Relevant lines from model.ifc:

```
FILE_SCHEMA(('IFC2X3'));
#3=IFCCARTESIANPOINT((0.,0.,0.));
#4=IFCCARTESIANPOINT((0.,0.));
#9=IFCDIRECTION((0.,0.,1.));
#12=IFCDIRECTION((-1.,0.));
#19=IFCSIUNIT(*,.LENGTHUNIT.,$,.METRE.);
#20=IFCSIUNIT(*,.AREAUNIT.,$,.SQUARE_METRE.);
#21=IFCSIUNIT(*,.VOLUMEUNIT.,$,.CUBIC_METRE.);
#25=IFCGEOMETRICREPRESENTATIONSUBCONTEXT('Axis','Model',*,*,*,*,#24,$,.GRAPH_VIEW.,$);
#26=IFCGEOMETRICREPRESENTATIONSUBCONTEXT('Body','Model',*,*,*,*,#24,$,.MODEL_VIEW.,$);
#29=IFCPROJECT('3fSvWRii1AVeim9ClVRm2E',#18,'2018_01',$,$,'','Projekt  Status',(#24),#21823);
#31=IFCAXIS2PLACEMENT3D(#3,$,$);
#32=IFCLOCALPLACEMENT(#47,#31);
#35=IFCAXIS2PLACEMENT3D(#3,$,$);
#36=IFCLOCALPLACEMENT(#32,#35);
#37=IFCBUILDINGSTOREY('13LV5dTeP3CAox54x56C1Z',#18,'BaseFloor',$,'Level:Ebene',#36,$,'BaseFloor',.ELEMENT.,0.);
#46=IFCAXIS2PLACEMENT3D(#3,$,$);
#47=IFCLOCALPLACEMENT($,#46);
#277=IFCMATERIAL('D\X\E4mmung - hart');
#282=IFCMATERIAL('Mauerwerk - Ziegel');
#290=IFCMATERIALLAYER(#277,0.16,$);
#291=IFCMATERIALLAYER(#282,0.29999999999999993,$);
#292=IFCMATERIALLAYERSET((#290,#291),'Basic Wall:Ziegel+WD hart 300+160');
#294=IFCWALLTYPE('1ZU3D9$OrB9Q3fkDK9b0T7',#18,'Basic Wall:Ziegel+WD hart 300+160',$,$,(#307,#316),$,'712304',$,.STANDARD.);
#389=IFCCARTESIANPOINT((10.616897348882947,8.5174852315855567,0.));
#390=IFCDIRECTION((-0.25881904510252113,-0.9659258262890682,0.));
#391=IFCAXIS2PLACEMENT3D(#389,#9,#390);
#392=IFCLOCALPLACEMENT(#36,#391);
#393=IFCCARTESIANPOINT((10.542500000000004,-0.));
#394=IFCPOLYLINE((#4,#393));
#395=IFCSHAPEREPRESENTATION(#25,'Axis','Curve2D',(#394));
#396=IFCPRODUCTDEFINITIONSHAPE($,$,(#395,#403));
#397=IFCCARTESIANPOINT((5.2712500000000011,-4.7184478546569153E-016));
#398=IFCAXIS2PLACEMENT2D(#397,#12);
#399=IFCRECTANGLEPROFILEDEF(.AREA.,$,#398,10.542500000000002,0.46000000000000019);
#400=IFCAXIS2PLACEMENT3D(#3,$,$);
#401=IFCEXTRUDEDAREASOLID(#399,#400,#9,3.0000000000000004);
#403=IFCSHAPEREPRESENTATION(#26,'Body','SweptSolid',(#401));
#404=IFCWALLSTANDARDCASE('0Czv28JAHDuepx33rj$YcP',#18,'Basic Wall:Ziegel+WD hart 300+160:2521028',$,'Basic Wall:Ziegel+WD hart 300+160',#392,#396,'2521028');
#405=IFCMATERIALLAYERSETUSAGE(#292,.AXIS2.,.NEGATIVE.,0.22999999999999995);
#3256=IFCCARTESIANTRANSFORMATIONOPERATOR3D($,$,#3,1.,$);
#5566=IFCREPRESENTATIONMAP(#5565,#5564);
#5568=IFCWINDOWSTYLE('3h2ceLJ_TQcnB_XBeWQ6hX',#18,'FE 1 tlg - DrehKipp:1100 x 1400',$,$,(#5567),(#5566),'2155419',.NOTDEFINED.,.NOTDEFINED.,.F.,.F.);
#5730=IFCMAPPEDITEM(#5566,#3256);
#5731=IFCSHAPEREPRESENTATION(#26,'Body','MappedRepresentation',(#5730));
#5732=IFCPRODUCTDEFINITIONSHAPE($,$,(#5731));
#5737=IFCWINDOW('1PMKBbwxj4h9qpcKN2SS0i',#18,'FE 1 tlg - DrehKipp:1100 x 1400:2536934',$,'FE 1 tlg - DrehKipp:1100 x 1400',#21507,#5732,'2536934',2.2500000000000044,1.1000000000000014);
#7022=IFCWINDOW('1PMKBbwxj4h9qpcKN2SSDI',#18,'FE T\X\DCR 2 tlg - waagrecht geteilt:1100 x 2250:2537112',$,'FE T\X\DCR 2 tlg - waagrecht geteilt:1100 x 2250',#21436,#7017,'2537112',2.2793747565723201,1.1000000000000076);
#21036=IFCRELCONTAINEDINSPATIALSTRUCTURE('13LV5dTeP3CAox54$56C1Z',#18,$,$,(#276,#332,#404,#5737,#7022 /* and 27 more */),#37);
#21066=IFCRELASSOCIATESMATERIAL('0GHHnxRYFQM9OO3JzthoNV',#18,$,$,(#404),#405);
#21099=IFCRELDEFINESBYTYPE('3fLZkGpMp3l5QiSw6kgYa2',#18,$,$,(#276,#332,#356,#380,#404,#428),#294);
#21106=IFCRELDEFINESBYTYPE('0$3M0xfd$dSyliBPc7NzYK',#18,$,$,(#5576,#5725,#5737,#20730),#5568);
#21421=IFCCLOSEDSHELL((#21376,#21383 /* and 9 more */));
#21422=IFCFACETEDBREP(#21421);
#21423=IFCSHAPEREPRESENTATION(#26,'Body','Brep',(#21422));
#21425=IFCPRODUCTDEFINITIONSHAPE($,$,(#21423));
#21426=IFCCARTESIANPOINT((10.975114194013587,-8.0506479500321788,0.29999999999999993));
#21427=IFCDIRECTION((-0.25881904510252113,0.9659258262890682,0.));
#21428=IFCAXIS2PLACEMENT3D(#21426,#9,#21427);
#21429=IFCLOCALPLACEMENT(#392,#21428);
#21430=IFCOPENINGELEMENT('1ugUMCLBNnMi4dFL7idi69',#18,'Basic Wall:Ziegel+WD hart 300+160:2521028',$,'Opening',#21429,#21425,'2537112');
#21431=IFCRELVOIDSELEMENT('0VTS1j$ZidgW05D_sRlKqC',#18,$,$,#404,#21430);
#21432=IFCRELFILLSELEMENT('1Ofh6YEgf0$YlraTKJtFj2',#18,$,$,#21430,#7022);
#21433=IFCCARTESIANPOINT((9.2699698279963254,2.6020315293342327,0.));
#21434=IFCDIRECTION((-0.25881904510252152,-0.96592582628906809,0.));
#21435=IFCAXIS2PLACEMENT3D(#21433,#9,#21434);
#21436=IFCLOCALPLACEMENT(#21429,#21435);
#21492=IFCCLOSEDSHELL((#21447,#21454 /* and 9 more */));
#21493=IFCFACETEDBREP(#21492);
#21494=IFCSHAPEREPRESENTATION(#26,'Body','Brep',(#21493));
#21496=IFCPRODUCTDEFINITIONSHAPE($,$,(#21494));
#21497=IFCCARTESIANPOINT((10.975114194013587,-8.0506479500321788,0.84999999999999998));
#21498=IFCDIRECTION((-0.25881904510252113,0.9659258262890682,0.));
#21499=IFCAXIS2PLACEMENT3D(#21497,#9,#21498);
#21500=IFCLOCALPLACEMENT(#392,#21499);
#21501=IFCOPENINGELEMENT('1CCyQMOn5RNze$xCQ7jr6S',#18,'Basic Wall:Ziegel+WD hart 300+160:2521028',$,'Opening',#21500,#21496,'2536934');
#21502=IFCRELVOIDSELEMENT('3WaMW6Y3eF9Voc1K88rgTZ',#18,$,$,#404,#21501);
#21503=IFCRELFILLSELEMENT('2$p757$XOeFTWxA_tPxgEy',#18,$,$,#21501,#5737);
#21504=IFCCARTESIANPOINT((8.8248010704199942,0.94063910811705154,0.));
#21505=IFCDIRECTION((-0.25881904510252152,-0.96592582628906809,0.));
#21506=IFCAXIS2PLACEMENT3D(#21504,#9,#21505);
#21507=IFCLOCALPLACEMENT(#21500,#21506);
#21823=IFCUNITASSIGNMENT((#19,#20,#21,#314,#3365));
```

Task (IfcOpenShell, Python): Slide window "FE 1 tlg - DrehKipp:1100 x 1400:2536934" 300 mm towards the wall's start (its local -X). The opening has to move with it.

```python
import ifcopenshell
import ifcopenshell.api.geometry
import ifcopenshell.util.placement

model = ifcopenshell.open("model.ifc")

window = model.by_id(5737)
opening = window.FillsVoids[0].RelatingOpeningElement
wall = opening.VoidsElements[0].RelatingBuildingElement

wall_matrix = ifcopenshell.util.placement.get_local_placement(wall.ObjectPlacement)
shift = wall_matrix[:3, 0] * -0.3
before = ifcopenshell.util.placement.get_local_placement(window.ObjectPlacement)[:3, 3].copy()

# The window is placed relative to its opening, so it follows when the opening moves.
matrix = ifcopenshell.util.placement.get_local_placement(opening.ObjectPlacement)
matrix[:3, 3] += shift
ifcopenshell.api.geometry.edit_object_placement(
    model, product=opening, matrix=matrix, is_si=False, should_transform_children=True
)

after = ifcopenshell.util.placement.get_local_placement(window.ObjectPlacement)[:3, 3]
print("window moved by", (after - before).round(3) + 0.0)

model.write("model_v2.ifc")
```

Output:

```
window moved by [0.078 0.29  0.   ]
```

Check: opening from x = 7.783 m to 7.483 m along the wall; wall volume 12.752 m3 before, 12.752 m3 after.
